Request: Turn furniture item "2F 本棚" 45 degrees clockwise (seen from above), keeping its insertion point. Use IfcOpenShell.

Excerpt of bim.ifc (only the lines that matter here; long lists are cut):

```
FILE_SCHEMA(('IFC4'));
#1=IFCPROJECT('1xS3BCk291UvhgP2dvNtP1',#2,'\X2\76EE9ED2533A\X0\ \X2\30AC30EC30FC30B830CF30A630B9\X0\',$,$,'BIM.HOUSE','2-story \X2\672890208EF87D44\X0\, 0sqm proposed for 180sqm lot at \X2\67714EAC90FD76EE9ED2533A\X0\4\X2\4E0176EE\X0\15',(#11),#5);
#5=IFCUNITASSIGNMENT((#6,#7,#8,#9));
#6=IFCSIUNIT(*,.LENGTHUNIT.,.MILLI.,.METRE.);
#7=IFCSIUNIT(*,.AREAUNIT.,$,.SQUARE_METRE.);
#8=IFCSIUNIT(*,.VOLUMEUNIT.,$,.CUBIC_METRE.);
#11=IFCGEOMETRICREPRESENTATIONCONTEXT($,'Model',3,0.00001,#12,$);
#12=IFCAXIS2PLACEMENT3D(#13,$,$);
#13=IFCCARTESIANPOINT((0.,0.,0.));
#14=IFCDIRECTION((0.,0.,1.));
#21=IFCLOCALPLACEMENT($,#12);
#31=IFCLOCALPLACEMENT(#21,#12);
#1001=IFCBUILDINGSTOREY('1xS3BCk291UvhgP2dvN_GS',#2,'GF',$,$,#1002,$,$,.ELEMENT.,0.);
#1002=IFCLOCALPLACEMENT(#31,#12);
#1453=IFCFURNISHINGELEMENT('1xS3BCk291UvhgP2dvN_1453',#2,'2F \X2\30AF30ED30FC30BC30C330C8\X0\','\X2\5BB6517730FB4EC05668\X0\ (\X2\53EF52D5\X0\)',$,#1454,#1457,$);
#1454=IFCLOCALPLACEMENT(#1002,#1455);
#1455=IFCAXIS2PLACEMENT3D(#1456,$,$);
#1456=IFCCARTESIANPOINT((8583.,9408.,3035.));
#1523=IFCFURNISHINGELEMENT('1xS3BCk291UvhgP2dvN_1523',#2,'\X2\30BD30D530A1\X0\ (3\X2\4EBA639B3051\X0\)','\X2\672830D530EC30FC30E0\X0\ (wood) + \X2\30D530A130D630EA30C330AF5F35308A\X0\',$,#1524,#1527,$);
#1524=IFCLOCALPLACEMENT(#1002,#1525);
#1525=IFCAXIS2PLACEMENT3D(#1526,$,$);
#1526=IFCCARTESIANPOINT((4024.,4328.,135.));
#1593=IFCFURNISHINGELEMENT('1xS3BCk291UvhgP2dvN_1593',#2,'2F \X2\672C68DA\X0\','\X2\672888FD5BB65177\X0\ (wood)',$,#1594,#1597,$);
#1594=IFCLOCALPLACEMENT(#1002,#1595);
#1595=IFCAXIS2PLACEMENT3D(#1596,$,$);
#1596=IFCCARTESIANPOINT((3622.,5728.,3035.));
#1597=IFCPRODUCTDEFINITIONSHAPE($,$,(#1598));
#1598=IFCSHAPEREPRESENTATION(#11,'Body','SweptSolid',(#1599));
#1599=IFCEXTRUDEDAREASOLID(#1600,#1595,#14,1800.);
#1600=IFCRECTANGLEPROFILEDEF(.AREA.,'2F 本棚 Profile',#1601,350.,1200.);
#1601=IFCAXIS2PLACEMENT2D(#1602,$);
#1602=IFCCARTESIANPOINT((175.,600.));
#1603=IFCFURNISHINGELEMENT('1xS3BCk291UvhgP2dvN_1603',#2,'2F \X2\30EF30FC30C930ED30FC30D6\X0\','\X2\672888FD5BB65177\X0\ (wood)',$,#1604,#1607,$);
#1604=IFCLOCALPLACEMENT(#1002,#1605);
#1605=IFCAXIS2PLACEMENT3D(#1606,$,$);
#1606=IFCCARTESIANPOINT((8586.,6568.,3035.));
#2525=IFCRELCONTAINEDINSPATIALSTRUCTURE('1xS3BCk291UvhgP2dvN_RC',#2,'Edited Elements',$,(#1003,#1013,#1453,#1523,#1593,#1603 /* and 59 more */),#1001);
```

```python
import ifcopenshell
import ifcopenshell.api.geometry
import ifcopenshell.util.placement

model = ifcopenshell.open("bim.ifc")

item = model.by_id(1593)
matrix = ifcopenshell.util.placement.get_local_placement(item.ObjectPlacement)
matrix = matrix @ ifcopenshell.util.placement.rotation(-45, "Z")
ifcopenshell.api.geometry.edit_object_placement(model, product=item, matrix=matrix, is_si=False)

print(ifcopenshell.util.placement.get_local_placement(item.ObjectPlacement).round(3) + 0.0)

model.write("bim_v2.ifc")
```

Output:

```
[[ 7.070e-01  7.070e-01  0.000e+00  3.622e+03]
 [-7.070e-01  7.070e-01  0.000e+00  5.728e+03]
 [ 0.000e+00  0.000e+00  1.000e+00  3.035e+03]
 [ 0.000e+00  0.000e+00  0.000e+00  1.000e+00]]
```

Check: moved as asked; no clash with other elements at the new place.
